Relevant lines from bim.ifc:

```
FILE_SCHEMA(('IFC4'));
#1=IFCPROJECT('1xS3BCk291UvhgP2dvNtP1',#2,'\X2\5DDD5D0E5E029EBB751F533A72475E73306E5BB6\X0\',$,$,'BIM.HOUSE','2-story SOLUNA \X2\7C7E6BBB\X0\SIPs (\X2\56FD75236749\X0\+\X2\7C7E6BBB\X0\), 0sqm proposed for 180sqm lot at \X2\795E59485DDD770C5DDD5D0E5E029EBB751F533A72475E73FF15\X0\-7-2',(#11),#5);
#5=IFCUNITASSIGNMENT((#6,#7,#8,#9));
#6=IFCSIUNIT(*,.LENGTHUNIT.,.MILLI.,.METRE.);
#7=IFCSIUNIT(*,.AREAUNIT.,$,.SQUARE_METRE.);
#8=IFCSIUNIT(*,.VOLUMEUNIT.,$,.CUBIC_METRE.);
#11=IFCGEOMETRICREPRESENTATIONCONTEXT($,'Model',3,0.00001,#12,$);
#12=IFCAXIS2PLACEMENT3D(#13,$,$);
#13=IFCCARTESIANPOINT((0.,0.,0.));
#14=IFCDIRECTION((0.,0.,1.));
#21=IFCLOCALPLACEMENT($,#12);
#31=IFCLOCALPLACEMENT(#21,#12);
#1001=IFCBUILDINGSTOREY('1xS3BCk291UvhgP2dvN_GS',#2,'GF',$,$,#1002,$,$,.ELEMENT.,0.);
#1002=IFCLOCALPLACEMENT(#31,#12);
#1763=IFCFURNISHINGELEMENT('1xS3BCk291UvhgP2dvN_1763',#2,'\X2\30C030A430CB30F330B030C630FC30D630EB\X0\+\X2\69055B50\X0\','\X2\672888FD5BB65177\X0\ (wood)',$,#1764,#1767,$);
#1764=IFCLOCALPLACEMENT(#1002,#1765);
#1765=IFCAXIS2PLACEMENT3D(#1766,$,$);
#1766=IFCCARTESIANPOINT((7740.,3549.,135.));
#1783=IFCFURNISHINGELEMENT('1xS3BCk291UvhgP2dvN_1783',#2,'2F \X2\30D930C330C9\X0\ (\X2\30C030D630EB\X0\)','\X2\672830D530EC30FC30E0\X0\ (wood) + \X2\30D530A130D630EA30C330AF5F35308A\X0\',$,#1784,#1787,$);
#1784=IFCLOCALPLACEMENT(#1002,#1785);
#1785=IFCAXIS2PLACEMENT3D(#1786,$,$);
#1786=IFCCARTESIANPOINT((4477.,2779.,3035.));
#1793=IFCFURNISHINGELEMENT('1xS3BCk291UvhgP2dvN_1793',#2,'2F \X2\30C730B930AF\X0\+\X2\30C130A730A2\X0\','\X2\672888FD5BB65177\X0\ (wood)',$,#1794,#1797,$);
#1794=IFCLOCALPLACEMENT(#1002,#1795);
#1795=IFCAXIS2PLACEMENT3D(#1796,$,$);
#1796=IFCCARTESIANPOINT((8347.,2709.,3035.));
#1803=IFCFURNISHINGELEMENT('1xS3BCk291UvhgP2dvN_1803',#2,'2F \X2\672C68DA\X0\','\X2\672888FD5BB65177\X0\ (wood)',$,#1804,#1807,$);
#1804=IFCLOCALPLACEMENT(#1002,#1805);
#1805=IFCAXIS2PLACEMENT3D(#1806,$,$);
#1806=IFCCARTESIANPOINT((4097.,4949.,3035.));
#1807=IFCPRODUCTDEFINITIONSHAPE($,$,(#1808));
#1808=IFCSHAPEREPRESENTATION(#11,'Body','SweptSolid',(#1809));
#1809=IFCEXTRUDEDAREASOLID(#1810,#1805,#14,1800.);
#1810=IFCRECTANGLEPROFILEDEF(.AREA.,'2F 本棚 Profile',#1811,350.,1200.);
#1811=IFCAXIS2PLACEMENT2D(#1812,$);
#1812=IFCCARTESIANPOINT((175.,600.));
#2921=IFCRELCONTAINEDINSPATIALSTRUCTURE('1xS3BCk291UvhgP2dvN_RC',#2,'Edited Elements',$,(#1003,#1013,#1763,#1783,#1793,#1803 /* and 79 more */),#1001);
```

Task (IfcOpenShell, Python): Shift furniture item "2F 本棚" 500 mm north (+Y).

```python
import ifcopenshell
import ifcopenshell.api.geometry
import ifcopenshell.util.placement

model = ifcopenshell.open("bim.ifc")

item = model.by_id(1803)
matrix = ifcopenshell.util.placement.get_local_placement(item.ObjectPlacement)
matrix[1, 3] += 500.0
ifcopenshell.api.geometry.edit_object_placement(model, product=item, matrix=matrix, is_si=False)

print(ifcopenshell.util.placement.get_local_placement(item.ObjectPlacement).round(3) + 0.0)

model.write("bim_rev.ifc")
```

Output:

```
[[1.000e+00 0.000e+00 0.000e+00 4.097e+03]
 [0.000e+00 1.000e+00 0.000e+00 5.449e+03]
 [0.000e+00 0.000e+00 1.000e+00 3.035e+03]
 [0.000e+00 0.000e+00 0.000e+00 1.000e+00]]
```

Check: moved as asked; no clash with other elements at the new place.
